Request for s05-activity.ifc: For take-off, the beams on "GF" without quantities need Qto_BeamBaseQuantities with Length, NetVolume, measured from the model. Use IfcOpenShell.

First a look at what the model holds.

```python
import ifcopenshell
import ifcopenshell.util.element
import ifcopenshell.util.unit

model = ifcopenshell.open("s05-activity.ifc")
print(model.schema)
for unit_type in ("LENGTHUNIT", "AREAUNIT", "VOLUMEUNIT"):
    print(unit_type, ifcopenshell.util.unit.calculate_unit_scale(model, unit_type))
storey = next(s for s in model.by_type("IfcBuildingStorey") if s.Name == "GF")
beams = [e for e in ifcopenshell.util.element.get_decomposition(storey) if e.is_a("IfcBeam")]
for e in sorted(beams, key=lambda e: e.id()):
    print(e.id(), e.is_a(), e.Name, list(ifcopenshell.util.element.get_psets(e, qtos_only=True)), sep=" | ")
```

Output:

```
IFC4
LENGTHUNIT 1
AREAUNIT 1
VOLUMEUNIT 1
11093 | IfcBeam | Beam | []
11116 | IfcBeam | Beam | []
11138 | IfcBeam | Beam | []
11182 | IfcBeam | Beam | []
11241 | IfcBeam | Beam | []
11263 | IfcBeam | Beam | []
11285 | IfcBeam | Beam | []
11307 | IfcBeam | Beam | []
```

```python
import ifcopenshell
import ifcopenshell.api.pset
import ifcopenshell.geom
import ifcopenshell.util.element
import ifcopenshell.util.shape
import ifcopenshell.util.unit

model = ifcopenshell.open("s05-activity.ifc")
unit_scale = ifcopenshell.util.unit.calculate_unit_scale(model)
volume_scale = ifcopenshell.util.unit.calculate_unit_scale(model, "VOLUMEUNIT")
settings = ifcopenshell.geom.settings()

storey = next(s for s in model.by_type("IfcBuildingStorey") if s.Name == "GF")
beams = [e for e in ifcopenshell.util.element.get_decomposition(storey) if e.is_a("IfcBeam")]

for e in sorted(beams, key=lambda e: e.id()):
    if ifcopenshell.util.element.get_psets(e, qtos_only=True, should_inherit=False):
        continue
    # Geometry comes back in metres, in the element's own axes.
    shape = ifcopenshell.geom.create_shape(settings, e)
    values = {
        "Length": ifcopenshell.util.shape.get_max_xyz(shape.geometry) / unit_scale,
        "NetVolume": ifcopenshell.util.shape.get_volume(shape.geometry) / volume_scale,
    }
    qto = ifcopenshell.api.pset.add_qto(model, product=e, name="Qto_BeamBaseQuantities")
    ifcopenshell.api.pset.edit_qto(model, qto=qto, properties=values)
    print(e.id(), {k: round(v, 3) for k, v in values.items()})

model.write("s05-activity_edited.ifc")
```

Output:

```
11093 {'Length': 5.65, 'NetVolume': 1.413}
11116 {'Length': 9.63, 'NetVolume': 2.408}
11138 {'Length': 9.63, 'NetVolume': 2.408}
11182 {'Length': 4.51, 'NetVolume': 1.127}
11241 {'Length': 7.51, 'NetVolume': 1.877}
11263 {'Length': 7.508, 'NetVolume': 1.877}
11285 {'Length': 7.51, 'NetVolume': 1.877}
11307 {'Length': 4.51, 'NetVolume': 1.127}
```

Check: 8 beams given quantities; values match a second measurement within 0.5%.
